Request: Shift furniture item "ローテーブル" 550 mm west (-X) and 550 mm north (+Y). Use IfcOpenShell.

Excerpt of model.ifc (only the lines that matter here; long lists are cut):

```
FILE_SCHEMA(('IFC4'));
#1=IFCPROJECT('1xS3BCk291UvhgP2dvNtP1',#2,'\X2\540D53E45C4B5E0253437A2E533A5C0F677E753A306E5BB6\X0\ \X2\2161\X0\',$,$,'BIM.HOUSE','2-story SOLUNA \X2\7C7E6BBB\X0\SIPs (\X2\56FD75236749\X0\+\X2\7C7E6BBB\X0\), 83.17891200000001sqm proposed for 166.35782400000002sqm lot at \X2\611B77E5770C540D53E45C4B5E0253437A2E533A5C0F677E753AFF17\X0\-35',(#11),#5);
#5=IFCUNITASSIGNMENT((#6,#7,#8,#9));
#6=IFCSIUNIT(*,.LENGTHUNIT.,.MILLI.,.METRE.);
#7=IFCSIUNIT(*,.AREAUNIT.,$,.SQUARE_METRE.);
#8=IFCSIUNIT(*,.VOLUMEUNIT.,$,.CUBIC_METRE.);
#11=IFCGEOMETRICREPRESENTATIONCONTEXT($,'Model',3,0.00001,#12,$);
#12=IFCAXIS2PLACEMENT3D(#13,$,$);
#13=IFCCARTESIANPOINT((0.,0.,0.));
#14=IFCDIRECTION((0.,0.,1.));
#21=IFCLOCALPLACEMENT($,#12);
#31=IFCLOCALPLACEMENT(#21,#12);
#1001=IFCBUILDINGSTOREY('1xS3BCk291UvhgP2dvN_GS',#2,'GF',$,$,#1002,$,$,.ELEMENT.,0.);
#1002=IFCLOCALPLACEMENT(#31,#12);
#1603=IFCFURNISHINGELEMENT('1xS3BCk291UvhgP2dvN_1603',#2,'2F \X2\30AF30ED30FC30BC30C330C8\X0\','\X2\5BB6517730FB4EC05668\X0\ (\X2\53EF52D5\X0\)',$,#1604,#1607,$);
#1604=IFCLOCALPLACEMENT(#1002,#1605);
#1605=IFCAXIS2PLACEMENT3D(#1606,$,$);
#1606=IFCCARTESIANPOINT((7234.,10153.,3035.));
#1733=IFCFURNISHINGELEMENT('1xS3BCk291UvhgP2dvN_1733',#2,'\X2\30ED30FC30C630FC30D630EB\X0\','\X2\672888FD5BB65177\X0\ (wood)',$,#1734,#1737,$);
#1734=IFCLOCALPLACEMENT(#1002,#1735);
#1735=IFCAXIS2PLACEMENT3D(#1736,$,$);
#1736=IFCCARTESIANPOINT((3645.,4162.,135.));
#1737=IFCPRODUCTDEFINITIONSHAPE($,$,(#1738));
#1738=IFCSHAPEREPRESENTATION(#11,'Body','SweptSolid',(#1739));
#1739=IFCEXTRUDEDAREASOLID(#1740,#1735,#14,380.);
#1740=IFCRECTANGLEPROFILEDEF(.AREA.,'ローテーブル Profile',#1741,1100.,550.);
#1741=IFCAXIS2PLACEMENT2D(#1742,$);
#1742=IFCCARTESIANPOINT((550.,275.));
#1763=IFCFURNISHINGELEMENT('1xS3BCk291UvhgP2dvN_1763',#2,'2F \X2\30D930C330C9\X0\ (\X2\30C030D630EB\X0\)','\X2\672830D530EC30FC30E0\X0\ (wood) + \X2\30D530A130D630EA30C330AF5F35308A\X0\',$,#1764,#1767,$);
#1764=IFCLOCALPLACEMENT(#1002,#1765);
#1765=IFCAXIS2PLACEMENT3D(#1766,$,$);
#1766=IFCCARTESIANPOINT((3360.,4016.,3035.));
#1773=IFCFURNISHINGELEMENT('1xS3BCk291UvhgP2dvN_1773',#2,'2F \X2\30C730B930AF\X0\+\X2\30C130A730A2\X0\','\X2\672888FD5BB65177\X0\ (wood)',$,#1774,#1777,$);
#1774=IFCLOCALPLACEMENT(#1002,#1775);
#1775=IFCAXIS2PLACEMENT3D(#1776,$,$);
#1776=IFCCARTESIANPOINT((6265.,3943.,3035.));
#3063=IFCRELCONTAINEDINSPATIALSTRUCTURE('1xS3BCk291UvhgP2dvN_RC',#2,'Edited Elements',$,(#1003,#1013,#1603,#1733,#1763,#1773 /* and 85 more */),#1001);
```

```python
import ifcopenshell
import ifcopenshell.api.geometry
import ifcopenshell.util.placement

model = ifcopenshell.open("model.ifc")

item = model.by_guid("1xS3BCk291UvhgP2dvN_1733")
matrix = ifcopenshell.util.placement.get_local_placement(item.ObjectPlacement)
matrix[0, 3] -= 550.0
matrix[1, 3] += 550.0
ifcopenshell.api.geometry.edit_object_placement(model, product=item, matrix=matrix, is_si=False)

print(ifcopenshell.util.placement.get_local_placement(item.ObjectPlacement).round(3) + 0.0)

model.write("model_edited.ifc")
```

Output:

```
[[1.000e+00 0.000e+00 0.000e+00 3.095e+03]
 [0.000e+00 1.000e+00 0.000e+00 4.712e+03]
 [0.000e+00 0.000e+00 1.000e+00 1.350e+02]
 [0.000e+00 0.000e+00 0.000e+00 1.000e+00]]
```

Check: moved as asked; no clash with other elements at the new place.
